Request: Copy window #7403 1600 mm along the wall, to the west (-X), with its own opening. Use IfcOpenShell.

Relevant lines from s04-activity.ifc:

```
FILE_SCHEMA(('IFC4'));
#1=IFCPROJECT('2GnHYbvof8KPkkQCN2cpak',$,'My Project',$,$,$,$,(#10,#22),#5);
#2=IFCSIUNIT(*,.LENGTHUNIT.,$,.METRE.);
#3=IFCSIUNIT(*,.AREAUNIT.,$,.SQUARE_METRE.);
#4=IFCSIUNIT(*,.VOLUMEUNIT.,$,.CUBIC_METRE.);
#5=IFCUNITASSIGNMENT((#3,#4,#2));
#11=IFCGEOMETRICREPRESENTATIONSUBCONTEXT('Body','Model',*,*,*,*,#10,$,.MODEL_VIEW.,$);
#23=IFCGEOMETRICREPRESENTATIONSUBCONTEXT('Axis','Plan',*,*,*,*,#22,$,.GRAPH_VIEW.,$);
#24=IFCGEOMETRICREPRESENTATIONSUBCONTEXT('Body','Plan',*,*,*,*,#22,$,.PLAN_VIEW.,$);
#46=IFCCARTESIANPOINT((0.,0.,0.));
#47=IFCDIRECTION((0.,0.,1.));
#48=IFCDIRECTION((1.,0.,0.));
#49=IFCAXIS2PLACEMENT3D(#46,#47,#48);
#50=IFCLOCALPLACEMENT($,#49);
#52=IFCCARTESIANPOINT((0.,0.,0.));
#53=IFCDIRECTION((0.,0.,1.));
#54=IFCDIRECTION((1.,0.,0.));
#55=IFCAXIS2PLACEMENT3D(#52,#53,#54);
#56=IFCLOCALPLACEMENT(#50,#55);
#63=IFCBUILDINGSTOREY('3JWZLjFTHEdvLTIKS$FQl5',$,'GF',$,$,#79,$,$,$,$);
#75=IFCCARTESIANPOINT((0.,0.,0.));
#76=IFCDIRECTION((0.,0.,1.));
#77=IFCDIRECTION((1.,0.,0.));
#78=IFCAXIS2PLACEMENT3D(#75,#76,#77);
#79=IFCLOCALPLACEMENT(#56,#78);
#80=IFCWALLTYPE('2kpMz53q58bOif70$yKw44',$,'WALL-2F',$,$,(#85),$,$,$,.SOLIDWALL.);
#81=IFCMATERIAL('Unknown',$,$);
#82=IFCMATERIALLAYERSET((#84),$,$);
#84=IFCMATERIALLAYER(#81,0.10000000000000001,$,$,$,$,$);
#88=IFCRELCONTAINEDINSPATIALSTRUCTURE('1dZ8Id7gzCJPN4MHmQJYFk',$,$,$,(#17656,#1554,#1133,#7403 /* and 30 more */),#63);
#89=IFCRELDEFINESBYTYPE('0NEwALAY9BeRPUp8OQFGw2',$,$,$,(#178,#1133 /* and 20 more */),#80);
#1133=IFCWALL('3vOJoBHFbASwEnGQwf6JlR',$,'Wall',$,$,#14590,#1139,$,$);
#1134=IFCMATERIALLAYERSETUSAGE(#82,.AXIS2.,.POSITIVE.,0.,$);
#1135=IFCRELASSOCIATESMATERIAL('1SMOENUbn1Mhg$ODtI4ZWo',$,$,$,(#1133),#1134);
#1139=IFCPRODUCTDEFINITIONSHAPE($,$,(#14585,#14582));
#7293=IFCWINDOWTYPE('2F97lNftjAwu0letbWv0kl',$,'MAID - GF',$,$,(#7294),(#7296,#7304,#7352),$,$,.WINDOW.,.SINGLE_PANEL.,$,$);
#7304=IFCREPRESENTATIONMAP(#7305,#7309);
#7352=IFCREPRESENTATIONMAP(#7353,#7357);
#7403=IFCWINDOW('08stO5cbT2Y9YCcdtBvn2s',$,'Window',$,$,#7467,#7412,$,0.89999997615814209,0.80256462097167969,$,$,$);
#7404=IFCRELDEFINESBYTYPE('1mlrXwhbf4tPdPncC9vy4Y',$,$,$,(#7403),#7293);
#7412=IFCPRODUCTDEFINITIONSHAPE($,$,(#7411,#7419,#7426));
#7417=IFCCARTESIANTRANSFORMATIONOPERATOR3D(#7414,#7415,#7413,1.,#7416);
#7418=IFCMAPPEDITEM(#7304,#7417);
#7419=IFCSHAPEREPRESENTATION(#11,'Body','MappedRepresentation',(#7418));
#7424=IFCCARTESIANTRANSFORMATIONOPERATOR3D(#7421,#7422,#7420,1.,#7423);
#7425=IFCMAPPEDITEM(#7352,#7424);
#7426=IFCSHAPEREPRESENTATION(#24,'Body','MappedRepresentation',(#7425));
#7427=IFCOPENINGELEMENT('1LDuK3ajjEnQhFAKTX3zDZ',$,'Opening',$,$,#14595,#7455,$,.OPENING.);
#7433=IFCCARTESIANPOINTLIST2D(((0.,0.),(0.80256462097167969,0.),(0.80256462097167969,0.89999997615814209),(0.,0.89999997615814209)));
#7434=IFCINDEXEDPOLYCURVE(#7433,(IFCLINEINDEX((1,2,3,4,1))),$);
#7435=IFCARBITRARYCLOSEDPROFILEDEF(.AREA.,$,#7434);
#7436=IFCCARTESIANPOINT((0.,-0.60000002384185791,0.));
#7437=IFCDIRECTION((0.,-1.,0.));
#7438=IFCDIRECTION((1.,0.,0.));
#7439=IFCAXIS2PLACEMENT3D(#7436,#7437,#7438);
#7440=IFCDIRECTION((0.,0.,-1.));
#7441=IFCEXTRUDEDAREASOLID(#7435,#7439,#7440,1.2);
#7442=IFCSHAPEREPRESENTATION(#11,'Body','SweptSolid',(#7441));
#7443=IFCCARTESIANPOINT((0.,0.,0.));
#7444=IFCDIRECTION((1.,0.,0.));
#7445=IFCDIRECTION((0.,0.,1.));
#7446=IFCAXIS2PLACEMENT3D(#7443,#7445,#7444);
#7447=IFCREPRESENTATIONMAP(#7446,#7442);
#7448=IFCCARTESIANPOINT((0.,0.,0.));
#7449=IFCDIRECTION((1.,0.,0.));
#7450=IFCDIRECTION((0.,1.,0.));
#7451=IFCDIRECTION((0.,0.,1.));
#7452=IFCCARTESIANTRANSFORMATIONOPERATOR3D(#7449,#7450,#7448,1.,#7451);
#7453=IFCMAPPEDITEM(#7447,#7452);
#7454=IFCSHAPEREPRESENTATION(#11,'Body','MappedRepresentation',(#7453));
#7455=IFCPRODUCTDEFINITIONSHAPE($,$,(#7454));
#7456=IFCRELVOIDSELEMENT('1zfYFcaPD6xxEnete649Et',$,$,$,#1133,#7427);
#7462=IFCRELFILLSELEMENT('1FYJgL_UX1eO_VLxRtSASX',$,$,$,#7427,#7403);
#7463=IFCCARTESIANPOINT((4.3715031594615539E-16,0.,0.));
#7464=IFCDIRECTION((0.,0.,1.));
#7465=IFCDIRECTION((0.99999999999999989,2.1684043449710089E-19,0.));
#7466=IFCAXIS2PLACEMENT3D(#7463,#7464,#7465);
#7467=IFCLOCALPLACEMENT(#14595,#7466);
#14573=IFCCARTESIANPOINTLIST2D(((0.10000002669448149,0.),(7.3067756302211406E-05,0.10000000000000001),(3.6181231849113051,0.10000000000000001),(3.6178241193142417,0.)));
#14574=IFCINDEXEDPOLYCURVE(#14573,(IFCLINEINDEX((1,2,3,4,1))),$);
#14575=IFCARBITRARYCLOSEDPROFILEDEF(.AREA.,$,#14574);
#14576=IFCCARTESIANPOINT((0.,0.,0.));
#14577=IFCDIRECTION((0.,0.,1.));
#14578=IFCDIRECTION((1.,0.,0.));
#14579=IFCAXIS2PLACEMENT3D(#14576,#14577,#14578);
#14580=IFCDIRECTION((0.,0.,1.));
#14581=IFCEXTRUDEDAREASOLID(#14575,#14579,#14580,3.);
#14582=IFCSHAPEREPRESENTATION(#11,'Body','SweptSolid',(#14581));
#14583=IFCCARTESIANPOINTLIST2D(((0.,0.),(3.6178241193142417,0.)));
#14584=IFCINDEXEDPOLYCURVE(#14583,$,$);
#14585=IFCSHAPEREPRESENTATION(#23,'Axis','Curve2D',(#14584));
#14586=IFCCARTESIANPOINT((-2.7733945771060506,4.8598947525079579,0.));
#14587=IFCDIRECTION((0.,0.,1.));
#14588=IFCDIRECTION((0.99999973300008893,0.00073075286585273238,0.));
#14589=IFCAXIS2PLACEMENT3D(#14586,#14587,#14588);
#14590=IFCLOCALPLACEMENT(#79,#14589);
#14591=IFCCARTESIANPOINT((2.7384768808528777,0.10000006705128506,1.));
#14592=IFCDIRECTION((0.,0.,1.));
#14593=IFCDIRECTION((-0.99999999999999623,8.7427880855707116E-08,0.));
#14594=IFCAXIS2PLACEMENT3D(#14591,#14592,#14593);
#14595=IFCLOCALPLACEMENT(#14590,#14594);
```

```python
import ifcopenshell
import ifcopenshell.api.feature
import ifcopenshell.api.geometry
import ifcopenshell.api.root
import ifcopenshell.geom
import ifcopenshell.util.element
import ifcopenshell.util.placement
import ifcopenshell.util.shape
import ifcopenshell.util.unit

model = ifcopenshell.open("s04-activity.ifc")
unit_scale = ifcopenshell.util.unit.calculate_unit_scale(model)
settings = ifcopenshell.geom.settings()


def volume(element):
    """Net volume in cubic metres, openings subtracted."""
    shape = ifcopenshell.geom.create_shape(settings, element)
    return ifcopenshell.util.shape.get_volume(shape.geometry)


window = model.by_guid("08stO5cbT2Y9YCcdtBvn2s")
opening = window.FillsVoids[0].RelatingOpeningElement
wall = opening.VoidsElements[0].RelatingBuildingElement
before = volume(wall)
shift = ifcopenshell.util.placement.get_local_placement(wall.ObjectPlacement)[:3, 0] * -1.6 / unit_scale

# copy_class copies the void relationship, type, container and properties, but no geometry.
new_opening = ifcopenshell.api.root.copy_class(model, product=opening)
new_opening.Representation = ifcopenshell.util.element.copy_deep(
    model, opening.Representation, exclude=["IfcGeometricRepresentationContext", "IfcRepresentationMap"]
)
new_window = ifcopenshell.api.root.copy_class(model, product=window)
new_window.Representation = ifcopenshell.util.element.copy_deep(
    model, window.Representation, exclude=["IfcGeometricRepresentationContext", "IfcRepresentationMap"]
)
ifcopenshell.api.feature.add_filling(model, opening=new_opening, element=new_window)

for old, new in ((opening, new_opening), (window, new_window)):
    matrix = ifcopenshell.util.placement.get_local_placement(old.ObjectPlacement)
    matrix[:3, 3] += shift
    ifcopenshell.api.geometry.edit_object_placement(model, product=new, matrix=matrix, is_si=False)

after = volume(wall)

print(f"wall volume {before:.3f} -> {after:.3f} m3")

model.write("s04-activity_edited.ifc")
```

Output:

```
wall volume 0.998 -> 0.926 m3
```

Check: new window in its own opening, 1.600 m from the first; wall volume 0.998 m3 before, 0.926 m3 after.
